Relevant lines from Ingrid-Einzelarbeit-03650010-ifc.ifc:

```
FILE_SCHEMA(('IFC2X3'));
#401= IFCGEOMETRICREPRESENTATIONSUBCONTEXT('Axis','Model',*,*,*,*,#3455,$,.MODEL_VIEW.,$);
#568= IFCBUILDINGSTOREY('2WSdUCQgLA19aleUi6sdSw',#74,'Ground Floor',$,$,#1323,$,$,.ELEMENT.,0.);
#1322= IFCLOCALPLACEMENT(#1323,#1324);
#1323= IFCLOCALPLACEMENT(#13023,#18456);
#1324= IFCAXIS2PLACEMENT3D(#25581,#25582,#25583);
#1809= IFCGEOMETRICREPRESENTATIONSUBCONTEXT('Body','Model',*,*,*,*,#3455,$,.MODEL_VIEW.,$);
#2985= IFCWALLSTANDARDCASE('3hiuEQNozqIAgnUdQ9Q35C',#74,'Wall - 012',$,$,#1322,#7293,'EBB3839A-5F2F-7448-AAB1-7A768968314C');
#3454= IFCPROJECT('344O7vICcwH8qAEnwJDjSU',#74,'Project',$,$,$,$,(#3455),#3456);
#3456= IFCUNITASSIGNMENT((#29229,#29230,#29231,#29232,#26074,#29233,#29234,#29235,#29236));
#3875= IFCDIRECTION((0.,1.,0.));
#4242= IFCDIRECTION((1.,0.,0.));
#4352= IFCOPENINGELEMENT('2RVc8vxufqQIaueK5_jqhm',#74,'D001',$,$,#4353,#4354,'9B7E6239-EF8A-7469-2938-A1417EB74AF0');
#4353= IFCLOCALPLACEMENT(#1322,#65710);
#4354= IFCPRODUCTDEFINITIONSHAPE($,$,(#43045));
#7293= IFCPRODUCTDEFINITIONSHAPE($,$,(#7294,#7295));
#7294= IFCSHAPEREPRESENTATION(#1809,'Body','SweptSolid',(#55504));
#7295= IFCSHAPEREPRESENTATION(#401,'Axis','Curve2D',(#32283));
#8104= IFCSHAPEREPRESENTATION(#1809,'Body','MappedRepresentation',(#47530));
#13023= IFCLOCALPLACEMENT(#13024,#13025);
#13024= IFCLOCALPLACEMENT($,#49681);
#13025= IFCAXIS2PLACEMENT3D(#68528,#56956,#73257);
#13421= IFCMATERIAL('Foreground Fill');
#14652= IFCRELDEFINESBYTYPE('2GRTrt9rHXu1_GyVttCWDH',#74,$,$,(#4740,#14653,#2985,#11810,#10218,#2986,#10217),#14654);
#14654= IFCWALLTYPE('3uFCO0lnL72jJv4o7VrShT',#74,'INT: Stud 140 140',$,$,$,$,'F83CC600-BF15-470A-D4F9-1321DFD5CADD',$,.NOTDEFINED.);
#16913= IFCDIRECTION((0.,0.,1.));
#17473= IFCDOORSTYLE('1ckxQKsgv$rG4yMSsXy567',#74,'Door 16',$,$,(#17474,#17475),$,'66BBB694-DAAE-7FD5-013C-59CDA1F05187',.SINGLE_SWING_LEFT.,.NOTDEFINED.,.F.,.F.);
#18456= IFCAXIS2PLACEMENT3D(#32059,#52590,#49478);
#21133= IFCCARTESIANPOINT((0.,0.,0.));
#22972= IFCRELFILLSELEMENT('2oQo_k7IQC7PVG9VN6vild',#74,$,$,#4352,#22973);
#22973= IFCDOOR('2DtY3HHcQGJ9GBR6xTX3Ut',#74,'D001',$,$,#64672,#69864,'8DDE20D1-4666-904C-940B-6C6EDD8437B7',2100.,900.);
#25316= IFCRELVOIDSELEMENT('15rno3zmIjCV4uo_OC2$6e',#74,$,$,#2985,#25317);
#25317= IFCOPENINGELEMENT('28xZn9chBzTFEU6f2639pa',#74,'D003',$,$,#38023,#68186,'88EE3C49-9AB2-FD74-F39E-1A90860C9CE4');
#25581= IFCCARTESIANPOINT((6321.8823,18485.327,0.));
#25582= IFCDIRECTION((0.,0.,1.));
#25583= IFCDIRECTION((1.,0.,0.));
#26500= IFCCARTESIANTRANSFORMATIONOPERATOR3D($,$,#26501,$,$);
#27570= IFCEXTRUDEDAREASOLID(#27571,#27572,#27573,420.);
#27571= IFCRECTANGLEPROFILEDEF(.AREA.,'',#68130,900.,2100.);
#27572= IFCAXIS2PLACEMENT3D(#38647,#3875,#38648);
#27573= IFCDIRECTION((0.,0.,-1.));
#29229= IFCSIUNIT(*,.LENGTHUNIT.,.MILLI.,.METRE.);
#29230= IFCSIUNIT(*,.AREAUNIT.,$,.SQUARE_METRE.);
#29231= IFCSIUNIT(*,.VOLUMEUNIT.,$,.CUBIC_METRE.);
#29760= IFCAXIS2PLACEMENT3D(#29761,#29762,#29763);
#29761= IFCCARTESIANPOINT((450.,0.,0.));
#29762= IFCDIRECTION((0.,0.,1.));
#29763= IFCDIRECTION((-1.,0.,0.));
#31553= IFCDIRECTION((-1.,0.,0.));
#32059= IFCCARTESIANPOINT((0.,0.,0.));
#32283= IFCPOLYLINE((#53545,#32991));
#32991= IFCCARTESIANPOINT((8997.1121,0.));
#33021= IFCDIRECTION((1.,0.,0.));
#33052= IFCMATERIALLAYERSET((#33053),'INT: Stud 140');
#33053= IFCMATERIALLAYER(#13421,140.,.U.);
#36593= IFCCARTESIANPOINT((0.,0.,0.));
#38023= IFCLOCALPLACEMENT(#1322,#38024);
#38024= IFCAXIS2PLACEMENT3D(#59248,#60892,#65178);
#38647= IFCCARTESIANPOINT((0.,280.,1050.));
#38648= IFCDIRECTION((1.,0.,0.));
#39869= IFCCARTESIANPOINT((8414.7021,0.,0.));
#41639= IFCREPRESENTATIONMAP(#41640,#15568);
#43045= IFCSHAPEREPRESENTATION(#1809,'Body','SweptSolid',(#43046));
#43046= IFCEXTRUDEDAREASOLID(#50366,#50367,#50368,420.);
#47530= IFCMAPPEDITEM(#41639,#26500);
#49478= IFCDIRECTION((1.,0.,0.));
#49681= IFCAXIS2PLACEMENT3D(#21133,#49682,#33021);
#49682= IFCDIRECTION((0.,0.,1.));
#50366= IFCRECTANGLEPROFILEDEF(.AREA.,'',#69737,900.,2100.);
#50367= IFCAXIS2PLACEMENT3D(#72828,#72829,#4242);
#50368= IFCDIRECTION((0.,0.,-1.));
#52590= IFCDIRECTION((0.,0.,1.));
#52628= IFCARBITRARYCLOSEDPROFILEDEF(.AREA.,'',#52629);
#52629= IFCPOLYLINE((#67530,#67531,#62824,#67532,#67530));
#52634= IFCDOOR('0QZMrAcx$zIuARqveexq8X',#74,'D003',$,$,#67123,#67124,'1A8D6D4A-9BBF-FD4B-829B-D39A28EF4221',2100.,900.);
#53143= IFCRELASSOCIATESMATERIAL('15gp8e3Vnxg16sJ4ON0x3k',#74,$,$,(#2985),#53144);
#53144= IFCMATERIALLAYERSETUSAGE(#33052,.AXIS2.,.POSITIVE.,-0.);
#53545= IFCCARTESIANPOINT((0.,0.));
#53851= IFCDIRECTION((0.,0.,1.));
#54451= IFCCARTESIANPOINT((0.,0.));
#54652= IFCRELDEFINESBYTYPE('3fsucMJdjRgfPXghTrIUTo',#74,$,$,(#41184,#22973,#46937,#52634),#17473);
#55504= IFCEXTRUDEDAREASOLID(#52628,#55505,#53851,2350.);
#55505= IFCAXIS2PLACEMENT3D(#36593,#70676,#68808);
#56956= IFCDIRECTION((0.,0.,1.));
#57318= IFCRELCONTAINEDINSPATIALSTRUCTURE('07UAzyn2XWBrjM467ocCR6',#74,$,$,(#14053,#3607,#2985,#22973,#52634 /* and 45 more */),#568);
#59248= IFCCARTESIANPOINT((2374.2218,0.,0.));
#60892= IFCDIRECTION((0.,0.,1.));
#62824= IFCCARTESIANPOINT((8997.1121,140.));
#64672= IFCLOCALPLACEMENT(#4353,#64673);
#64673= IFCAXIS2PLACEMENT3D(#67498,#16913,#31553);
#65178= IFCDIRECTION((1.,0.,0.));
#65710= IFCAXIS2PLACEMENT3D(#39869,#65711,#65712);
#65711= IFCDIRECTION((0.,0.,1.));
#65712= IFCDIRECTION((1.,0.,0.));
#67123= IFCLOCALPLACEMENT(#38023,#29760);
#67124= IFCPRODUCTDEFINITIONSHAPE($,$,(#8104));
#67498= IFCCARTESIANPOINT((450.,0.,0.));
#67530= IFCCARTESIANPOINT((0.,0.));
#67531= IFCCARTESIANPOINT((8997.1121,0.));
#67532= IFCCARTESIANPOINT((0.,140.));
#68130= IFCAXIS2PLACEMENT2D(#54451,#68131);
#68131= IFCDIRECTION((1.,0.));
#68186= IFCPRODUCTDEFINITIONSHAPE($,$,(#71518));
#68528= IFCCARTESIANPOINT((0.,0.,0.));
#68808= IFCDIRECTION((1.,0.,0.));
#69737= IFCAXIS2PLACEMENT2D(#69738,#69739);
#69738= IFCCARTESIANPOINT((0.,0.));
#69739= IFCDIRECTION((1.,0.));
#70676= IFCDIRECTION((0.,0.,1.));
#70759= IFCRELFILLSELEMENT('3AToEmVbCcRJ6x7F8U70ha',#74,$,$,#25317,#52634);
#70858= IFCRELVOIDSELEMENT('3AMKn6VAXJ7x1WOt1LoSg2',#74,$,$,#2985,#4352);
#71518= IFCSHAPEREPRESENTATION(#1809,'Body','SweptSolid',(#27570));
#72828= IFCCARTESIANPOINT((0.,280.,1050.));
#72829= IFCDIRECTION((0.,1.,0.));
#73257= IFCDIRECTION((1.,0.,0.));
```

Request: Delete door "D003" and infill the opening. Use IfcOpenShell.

```python
import ifcopenshell
import ifcopenshell.api.feature
import ifcopenshell.api.root
import ifcopenshell.geom
import ifcopenshell.util.shape

model = ifcopenshell.open("Ingrid-Einzelarbeit-03650010-ifc.ifc")
settings = ifcopenshell.geom.settings()


def volume(element):
    """Net volume in cubic metres, openings subtracted."""
    shape = ifcopenshell.geom.create_shape(settings, element)
    return ifcopenshell.util.shape.get_volume(shape.geometry)


door = model.by_guid("0QZMrAcx$zIuARqveexq8X")
opening = door.FillsVoids[0].RelatingOpeningElement
wall = opening.VoidsElements[0].RelatingBuildingElement
before = volume(wall)

ifcopenshell.api.root.remove_product(model, product=door)
ifcopenshell.api.feature.remove_feature(model, feature=opening)

after = volume(wall)

print(f"wall volume {before:.3f} -> {after:.3f} m3")

model.write("Ingrid-Einzelarbeit-03650010-ifc_updated.ifc")
```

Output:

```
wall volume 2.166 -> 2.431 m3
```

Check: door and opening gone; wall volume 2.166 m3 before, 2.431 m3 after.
